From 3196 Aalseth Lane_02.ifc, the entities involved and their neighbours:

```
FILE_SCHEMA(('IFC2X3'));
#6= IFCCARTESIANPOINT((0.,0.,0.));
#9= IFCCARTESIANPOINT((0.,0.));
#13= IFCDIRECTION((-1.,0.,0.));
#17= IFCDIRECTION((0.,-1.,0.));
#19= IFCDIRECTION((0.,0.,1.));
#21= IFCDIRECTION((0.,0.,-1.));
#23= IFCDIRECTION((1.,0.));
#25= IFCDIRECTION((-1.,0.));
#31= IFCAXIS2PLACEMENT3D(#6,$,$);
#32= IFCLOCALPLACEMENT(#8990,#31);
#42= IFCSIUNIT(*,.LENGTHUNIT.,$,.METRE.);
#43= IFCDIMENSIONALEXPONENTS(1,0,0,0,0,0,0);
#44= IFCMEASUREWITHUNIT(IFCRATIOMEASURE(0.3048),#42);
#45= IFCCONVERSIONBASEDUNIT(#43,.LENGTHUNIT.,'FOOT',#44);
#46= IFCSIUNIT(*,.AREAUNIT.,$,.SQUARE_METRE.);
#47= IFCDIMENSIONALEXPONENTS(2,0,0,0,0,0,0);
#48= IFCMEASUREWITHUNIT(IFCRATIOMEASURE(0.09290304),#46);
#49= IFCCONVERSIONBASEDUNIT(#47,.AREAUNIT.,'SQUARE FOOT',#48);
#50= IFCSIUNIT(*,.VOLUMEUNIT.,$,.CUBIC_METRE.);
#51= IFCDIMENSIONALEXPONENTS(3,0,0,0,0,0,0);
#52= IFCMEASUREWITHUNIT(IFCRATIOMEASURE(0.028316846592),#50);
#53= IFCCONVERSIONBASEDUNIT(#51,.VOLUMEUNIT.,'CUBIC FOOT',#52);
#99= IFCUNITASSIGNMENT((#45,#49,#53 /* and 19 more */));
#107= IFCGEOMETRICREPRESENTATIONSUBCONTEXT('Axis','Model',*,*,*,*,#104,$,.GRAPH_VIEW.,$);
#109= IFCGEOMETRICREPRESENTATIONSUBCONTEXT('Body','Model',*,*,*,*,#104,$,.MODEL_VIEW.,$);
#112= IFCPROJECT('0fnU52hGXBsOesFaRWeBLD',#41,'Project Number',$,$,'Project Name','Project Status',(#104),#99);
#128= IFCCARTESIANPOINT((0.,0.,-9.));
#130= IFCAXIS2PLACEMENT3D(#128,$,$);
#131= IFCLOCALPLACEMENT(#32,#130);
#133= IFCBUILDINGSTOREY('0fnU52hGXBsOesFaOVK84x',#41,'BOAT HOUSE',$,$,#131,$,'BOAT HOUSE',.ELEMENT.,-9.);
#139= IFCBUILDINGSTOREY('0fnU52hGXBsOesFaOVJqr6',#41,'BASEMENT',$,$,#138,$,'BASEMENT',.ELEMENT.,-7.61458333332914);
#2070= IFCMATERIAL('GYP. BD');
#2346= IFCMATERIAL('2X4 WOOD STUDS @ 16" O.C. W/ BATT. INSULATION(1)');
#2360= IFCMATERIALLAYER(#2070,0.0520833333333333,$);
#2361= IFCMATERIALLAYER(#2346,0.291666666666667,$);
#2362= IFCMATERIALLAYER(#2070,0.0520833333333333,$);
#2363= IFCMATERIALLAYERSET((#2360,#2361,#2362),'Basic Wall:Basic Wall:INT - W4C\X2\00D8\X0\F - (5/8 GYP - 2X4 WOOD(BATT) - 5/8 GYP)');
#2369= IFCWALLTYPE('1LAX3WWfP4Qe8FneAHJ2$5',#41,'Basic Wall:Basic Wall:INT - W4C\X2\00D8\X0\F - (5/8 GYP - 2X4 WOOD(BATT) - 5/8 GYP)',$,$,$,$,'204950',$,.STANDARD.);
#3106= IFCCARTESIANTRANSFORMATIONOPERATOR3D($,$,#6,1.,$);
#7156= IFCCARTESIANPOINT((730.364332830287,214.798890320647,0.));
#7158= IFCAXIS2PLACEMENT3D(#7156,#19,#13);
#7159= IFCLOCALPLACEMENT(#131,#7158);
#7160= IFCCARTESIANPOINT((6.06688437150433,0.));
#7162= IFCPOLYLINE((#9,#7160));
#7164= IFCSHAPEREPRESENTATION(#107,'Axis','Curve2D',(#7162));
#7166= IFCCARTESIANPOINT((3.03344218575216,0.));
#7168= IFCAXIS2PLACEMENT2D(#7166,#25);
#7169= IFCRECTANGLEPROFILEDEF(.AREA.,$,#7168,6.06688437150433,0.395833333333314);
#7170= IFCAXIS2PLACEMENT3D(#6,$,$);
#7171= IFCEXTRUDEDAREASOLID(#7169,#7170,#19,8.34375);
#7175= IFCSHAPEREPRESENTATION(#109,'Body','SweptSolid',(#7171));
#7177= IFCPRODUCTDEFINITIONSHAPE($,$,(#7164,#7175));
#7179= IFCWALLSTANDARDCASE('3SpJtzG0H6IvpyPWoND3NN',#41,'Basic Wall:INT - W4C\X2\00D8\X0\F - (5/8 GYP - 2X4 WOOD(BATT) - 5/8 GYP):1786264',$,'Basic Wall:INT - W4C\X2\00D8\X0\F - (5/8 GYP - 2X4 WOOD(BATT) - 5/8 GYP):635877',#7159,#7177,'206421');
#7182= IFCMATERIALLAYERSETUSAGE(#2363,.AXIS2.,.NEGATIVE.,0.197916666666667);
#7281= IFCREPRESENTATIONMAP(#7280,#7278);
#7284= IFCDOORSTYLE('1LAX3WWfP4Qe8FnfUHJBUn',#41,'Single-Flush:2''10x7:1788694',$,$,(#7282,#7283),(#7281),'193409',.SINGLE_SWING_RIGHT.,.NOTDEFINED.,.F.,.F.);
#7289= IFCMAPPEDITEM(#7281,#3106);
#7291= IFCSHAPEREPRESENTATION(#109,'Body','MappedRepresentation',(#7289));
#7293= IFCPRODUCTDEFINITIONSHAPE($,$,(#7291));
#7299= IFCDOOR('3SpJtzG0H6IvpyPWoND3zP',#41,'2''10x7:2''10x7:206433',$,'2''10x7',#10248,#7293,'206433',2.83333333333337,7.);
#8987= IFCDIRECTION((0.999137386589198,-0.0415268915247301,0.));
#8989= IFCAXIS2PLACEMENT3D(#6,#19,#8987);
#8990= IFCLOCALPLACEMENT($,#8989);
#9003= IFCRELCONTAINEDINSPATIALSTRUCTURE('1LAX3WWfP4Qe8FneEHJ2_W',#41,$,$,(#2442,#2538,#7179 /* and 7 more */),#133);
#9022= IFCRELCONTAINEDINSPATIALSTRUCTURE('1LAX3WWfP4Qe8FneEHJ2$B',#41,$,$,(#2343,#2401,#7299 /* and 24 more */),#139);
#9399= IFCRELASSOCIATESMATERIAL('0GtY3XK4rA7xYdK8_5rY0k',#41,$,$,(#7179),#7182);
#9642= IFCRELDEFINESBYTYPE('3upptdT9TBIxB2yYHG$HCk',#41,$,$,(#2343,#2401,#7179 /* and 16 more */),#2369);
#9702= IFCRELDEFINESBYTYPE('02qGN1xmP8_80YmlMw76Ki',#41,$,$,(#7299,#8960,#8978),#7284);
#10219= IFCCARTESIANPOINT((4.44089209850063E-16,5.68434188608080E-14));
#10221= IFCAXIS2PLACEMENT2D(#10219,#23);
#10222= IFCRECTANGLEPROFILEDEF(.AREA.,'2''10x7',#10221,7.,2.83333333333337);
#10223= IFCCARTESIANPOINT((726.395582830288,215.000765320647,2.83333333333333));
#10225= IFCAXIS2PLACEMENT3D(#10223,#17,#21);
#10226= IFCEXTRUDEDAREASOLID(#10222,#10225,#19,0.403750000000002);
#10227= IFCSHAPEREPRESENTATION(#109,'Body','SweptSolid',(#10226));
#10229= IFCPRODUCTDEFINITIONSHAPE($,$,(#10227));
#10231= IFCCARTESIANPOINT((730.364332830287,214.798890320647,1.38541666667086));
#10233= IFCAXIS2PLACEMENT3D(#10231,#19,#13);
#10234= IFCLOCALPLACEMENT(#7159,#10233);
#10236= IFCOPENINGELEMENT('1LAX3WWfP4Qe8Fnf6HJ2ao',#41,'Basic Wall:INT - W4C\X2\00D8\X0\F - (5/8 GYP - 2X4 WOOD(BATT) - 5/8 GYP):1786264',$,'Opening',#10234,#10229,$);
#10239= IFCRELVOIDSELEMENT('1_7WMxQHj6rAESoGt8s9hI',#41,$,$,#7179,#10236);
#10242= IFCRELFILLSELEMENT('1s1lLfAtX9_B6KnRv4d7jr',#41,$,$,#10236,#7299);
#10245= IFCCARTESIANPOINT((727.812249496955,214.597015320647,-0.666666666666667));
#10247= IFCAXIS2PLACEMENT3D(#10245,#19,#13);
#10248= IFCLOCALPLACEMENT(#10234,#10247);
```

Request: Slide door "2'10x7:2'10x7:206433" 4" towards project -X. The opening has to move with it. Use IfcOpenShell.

```python
import ifcopenshell
import ifcopenshell.api.geometry
import ifcopenshell.util.placement
import ifcopenshell.util.unit

model = ifcopenshell.open("3196 Aalseth Lane_02.ifc")
unit_scale = ifcopenshell.util.unit.calculate_unit_scale(model)

door = model.by_guid("3SpJtzG0H6IvpyPWoND3zP")
opening = door.FillsVoids[0].RelatingOpeningElement
wall = opening.VoidsElements[0].RelatingBuildingElement

wall_matrix = ifcopenshell.util.placement.get_local_placement(wall.ObjectPlacement)
shift = wall_matrix[:3, 0] * 4 * 0.0254 / unit_scale
before = ifcopenshell.util.placement.get_local_placement(door.ObjectPlacement)[:3, 3].copy()

# The door is placed relative to its opening, so it follows when the opening moves.
matrix = ifcopenshell.util.placement.get_local_placement(opening.ObjectPlacement)
matrix[:3, 3] += shift
ifcopenshell.api.geometry.edit_object_placement(
    model, product=opening, matrix=matrix, is_si=False, should_transform_children=True
)

after = ifcopenshell.util.placement.get_local_placement(door.ObjectPlacement)[:3, 3]
print("door moved by", (after - before).round(3) + 0.0)

model.write("3196 Aalseth Lane_02_rev.ifc")
```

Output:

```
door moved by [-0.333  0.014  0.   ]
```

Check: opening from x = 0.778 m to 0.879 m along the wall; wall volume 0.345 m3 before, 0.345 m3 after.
